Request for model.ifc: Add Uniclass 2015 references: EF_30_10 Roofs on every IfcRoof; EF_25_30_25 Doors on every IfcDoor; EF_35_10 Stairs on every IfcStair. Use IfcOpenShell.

First a look at what the model holds.

```python
import ifcopenshell

model = ifcopenshell.open("model.ifc")
print(model.schema)
print("classifications:", [c.Name for c in model.by_type("IfcClassification")])
for ifc_class in ("IfcDoor", "IfcRoof", "IfcStair", "IfcWall", "IfcWindow"):
    print(ifc_class, len(model.by_type(ifc_class)))
```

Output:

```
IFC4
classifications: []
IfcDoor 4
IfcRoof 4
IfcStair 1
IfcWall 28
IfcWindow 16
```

```python
import ifcopenshell
import ifcopenshell.api.classification

model = ifcopenshell.open("model.ifc")

system = ifcopenshell.api.classification.add_classification(model, classification="Uniclass 2015")

codes = {
    "IfcRoof": ("EF_30_10", "Roofs"),
    "IfcDoor": ("EF_25_30_25", "Doors"),
    "IfcStair": ("EF_35_10", "Stairs"),
}
for ifc_class, (code, name) in codes.items():
    products = model.by_type(ifc_class)
    ifcopenshell.api.classification.add_reference(
        model, products=products, classification=system, identification=code, name=name
    )
    print(code, len(products))

model.write("model_rev.ifc")
```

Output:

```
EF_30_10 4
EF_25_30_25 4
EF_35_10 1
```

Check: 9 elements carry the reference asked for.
